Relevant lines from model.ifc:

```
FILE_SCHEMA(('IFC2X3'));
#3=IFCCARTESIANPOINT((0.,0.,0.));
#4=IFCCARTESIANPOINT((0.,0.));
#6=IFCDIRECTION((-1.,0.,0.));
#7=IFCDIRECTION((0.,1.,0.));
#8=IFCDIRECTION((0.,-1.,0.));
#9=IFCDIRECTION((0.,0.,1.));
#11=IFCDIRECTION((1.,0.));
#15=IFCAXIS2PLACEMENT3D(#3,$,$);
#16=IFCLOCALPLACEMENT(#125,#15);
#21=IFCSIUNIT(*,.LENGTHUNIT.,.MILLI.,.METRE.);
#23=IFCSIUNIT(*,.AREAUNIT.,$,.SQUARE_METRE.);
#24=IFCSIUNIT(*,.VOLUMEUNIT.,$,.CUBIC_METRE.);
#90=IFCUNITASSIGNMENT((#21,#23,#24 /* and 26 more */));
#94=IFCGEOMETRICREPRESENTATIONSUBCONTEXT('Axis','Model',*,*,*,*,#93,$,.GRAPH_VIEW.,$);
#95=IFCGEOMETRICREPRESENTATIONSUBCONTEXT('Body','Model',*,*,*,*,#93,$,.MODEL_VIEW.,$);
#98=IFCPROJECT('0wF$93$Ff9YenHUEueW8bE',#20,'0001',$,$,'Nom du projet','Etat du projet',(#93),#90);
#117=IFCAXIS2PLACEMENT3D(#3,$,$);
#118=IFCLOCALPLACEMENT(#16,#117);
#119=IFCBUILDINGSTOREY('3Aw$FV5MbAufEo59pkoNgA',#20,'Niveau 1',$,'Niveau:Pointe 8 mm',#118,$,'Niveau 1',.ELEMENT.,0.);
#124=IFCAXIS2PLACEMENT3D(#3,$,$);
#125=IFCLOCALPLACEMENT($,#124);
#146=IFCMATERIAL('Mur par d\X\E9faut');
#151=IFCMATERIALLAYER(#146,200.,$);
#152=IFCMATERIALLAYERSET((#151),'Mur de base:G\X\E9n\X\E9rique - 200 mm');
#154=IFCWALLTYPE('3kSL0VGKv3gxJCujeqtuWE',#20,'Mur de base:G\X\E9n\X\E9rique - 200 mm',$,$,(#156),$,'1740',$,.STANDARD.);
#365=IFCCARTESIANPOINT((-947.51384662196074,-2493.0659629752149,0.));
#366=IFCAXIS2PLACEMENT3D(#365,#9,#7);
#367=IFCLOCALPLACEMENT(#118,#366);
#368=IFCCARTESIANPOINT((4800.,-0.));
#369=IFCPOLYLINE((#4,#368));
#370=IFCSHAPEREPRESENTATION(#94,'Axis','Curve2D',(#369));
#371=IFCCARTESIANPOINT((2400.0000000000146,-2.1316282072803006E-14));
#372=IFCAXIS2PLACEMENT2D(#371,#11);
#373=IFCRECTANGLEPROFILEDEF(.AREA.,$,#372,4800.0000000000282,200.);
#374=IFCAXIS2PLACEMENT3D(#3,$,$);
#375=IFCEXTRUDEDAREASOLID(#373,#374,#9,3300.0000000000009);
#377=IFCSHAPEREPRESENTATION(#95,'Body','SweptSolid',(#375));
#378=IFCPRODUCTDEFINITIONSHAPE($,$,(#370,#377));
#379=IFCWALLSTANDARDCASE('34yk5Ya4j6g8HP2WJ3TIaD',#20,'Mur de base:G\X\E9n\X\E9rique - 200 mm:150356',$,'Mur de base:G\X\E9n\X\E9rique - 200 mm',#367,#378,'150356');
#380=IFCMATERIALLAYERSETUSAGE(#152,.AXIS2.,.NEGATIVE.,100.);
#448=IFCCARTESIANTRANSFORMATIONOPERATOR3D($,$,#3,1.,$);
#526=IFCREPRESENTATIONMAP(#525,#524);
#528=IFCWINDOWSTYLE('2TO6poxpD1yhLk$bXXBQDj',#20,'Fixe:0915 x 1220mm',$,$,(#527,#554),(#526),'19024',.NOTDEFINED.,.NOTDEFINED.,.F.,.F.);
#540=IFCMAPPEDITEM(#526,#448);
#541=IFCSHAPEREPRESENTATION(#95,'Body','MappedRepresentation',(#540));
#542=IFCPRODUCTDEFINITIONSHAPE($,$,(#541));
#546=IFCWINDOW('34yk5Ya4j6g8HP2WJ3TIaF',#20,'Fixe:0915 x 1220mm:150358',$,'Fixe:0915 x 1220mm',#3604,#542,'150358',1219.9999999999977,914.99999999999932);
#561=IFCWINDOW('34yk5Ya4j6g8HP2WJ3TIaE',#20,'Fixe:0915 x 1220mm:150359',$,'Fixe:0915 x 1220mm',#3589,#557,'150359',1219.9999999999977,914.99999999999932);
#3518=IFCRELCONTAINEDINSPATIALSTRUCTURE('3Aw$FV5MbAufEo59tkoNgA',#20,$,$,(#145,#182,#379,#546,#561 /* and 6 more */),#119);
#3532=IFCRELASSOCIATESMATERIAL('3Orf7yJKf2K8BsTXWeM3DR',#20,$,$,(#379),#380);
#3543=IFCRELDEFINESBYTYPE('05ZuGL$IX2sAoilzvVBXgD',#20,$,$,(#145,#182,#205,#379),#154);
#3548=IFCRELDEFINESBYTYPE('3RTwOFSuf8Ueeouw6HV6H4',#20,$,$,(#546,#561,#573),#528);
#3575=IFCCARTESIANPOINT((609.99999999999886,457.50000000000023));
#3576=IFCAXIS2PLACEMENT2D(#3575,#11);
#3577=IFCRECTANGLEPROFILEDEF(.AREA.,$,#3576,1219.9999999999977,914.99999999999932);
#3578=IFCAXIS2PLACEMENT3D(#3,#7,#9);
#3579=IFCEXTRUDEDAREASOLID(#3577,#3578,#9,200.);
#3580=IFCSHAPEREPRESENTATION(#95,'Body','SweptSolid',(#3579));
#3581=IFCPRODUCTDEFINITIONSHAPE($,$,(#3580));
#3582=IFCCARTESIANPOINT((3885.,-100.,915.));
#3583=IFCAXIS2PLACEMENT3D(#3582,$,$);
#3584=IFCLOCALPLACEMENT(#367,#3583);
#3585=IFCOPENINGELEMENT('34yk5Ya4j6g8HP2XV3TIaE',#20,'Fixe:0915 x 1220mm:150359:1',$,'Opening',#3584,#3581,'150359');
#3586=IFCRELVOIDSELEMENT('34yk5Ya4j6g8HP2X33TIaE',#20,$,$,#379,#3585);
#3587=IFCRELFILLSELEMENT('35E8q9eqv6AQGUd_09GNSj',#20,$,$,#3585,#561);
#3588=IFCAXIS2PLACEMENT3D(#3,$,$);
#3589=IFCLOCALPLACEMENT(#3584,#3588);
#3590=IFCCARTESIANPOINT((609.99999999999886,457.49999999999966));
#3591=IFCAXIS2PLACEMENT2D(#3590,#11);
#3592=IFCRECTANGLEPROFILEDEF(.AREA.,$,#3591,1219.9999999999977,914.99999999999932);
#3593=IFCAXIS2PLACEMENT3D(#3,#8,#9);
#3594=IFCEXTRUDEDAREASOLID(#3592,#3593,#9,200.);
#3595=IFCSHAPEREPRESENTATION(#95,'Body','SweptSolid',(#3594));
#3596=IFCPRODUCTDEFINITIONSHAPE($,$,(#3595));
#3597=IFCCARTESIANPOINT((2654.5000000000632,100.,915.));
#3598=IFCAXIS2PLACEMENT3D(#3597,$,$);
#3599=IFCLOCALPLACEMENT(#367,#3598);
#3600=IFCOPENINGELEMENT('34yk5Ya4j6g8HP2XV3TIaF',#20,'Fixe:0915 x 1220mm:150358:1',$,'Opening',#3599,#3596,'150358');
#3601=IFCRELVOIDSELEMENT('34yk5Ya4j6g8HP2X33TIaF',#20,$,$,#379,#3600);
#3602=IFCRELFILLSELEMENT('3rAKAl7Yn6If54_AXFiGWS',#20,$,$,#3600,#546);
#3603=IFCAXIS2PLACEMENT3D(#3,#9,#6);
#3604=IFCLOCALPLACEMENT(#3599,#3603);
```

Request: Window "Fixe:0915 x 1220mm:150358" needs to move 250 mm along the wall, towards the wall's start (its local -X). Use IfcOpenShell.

```python
import ifcopenshell
import ifcopenshell.api.geometry
import ifcopenshell.util.placement
import ifcopenshell.util.unit

model = ifcopenshell.open("model.ifc")
unit_scale = ifcopenshell.util.unit.calculate_unit_scale(model)

window = model.by_guid("34yk5Ya4j6g8HP2WJ3TIaF")
opening = window.FillsVoids[0].RelatingOpeningElement
wall = opening.VoidsElements[0].RelatingBuildingElement

wall_matrix = ifcopenshell.util.placement.get_local_placement(wall.ObjectPlacement)
shift = wall_matrix[:3, 0] * -0.25 / unit_scale
before = ifcopenshell.util.placement.get_local_placement(window.ObjectPlacement)[:3, 3].copy()

# The window is placed relative to its opening, so it follows when the opening moves.
matrix = ifcopenshell.util.placement.get_local_placement(opening.ObjectPlacement)
matrix[:3, 3] += shift
ifcopenshell.api.geometry.edit_object_placement(
    model, product=opening, matrix=matrix, is_si=False, should_transform_children=True
)

after = ifcopenshell.util.placement.get_local_placement(window.ObjectPlacement)[:3, 3]
print("window moved by", (after - before).round(3) + 0.0)

model.write("model_updated.ifc")
```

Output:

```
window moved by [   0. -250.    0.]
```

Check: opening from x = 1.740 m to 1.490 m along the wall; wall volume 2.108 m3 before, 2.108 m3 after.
